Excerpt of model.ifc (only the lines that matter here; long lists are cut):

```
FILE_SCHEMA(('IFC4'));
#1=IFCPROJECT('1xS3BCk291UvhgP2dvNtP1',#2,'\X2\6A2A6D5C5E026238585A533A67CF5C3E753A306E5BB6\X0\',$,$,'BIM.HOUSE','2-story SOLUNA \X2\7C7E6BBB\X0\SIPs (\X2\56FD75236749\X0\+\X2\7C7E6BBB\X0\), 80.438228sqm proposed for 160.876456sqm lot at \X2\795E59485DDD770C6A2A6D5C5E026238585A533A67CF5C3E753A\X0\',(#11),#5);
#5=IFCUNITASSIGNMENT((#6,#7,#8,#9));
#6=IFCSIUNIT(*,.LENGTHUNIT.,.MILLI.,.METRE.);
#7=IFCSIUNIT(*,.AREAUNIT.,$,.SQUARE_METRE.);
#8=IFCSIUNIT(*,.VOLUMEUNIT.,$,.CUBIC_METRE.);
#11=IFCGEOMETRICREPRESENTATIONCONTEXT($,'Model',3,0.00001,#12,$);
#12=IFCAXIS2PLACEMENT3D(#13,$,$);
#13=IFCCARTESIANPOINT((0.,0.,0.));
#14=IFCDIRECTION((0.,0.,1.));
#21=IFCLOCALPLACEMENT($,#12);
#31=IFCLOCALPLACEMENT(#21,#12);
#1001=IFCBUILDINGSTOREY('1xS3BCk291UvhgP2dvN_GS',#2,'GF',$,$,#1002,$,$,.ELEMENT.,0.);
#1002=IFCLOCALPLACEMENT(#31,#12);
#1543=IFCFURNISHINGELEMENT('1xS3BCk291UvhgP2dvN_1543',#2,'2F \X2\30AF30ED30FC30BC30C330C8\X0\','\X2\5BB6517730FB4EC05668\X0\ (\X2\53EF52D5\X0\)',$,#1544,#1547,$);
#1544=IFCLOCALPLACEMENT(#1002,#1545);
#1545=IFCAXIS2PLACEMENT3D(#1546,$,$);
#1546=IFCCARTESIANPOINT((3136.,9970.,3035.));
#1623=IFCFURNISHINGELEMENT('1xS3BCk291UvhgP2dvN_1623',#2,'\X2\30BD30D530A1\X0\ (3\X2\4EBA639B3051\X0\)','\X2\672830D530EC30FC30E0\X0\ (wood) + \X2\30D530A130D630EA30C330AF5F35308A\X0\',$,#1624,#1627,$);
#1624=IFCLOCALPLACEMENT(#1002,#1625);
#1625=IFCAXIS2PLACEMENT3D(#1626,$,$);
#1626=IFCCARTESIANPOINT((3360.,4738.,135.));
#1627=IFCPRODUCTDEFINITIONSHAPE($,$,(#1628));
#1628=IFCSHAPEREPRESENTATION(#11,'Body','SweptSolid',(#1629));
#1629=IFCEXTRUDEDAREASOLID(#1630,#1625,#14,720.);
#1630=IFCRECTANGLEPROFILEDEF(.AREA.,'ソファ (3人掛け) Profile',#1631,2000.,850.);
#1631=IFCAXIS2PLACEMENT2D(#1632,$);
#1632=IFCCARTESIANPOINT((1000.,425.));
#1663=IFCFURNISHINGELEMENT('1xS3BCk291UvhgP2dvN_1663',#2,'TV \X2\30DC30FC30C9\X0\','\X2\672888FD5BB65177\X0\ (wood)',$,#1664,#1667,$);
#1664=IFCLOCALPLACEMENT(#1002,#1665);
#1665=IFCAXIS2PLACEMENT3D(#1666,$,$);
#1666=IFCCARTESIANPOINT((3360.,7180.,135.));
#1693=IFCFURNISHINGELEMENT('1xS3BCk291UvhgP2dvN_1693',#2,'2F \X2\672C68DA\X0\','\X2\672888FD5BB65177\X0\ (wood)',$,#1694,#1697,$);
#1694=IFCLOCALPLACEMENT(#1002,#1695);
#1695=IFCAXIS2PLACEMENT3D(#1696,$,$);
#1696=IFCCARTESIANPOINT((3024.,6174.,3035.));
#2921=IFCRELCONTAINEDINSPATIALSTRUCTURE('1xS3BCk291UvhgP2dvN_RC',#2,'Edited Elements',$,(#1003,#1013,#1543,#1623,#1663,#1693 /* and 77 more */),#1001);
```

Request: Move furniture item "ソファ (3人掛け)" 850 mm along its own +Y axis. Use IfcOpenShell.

```python
import ifcopenshell
import ifcopenshell.api.geometry
import ifcopenshell.util.placement

model = ifcopenshell.open("model.ifc")

item = model.by_guid("1xS3BCk291UvhgP2dvN_1623")
matrix = ifcopenshell.util.placement.get_local_placement(item.ObjectPlacement)
matrix[:3, 3] += matrix[:3, 1] * 850.0
ifcopenshell.api.geometry.edit_object_placement(model, product=item, matrix=matrix, is_si=False)

print(ifcopenshell.util.placement.get_local_placement(item.ObjectPlacement).round(3) + 0.0)

model.write("model_updated.ifc")
```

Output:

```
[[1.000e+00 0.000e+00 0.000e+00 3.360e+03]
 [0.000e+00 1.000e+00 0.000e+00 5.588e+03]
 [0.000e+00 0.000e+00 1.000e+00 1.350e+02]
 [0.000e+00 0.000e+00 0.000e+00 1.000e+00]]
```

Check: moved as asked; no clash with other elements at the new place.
